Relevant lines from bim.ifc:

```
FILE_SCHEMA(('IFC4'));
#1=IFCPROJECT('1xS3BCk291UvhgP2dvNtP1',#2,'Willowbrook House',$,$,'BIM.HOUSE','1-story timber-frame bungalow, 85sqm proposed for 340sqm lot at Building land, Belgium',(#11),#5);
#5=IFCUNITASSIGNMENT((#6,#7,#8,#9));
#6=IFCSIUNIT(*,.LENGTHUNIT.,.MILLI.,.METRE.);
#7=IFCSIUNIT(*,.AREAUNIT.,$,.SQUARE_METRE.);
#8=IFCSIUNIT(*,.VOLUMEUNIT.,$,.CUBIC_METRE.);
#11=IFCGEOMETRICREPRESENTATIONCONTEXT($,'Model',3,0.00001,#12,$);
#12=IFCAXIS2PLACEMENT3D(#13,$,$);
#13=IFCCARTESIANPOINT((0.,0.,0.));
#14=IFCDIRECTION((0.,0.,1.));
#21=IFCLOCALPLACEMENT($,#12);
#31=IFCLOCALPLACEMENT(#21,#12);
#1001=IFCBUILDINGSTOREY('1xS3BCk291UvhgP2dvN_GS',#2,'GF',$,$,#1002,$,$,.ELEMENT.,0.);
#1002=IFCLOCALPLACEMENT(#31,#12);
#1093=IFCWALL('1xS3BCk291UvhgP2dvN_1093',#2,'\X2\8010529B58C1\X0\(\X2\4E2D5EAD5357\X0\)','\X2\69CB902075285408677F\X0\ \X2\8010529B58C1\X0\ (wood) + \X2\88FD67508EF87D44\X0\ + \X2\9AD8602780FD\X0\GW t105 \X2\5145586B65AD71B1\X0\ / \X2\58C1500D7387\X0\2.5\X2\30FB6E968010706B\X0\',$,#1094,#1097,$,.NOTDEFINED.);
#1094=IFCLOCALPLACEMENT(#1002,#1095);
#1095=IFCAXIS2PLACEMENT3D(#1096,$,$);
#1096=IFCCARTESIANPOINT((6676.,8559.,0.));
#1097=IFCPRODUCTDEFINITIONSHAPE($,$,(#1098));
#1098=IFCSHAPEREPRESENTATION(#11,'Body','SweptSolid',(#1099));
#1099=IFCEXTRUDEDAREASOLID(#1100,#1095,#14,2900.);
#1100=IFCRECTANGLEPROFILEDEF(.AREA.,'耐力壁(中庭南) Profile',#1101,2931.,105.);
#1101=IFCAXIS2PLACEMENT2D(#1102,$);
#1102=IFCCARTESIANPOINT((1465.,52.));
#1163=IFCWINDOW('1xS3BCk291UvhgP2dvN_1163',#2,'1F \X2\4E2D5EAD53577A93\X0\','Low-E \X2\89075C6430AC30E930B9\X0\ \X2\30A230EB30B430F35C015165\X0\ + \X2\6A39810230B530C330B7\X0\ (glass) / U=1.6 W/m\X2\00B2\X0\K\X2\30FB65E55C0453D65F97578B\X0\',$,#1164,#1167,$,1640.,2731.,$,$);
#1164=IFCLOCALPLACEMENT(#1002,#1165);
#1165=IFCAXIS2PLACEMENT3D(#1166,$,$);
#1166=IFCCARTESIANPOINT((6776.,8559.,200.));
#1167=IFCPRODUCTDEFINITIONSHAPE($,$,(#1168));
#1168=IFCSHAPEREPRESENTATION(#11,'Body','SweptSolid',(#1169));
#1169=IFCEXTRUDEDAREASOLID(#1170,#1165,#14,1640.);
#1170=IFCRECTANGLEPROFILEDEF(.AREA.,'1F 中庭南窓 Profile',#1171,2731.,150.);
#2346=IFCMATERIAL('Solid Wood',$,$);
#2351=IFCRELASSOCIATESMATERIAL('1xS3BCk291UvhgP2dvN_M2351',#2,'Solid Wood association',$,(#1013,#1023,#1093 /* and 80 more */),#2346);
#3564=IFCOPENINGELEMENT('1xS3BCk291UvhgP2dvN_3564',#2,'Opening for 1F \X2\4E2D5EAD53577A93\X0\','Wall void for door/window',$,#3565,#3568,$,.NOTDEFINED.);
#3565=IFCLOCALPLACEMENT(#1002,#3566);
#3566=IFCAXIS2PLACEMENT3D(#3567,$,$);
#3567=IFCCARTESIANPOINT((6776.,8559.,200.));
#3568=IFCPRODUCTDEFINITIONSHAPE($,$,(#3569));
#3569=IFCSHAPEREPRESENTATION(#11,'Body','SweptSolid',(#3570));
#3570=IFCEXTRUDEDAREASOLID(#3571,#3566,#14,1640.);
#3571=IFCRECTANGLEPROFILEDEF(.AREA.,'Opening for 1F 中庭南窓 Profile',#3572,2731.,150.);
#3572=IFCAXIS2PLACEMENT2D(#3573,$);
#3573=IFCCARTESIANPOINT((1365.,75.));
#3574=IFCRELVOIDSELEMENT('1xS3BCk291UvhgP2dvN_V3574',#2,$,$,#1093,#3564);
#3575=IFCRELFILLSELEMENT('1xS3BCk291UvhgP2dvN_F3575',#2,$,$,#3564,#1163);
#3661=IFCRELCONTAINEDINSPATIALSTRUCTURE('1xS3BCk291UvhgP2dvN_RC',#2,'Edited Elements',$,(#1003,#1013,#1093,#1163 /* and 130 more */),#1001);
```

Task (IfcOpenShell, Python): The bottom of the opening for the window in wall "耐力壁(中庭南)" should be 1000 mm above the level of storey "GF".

```python
import numpy as np
import ifcopenshell
import ifcopenshell.api.geometry
import ifcopenshell.geom
import ifcopenshell.util.element
import ifcopenshell.util.placement
import ifcopenshell.util.shape
import ifcopenshell.util.unit

model = ifcopenshell.open("bim.ifc")
unit_scale = ifcopenshell.util.unit.calculate_unit_scale(model)

window = model.by_guid("1xS3BCk291UvhgP2dvN_1163")
opening = window.FillsVoids[0].RelatingOpeningElement
storey = ifcopenshell.util.element.get_container(window, ifc_class="IfcBuildingStorey")
level = ifcopenshell.util.placement.get_local_placement(storey.ObjectPlacement)[2, 3]

# The opening's origin need not be at the sill, so measure its lowest point.
shape = ifcopenshell.geom.create_shape(ifcopenshell.geom.settings(), opening)
bottom = ifcopenshell.util.shape.get_shape_bottom_elevation(shape, shape.geometry) / unit_scale
dz = level + 1 / unit_scale - bottom

shift = np.array([0.0, 0.0, dz])
# The window is not placed relative to its opening, so move both.
for product in (opening, window):
    matrix = ifcopenshell.util.placement.get_local_placement(product.ObjectPlacement)
    matrix[:3, 3] += shift
    ifcopenshell.api.geometry.edit_object_placement(model, product=product, matrix=matrix, is_si=False)

print(f"moved by {dz * unit_scale:+.3f} m")

model.write("bim-out.ifc")
```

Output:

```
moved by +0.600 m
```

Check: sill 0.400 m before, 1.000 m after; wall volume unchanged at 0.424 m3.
